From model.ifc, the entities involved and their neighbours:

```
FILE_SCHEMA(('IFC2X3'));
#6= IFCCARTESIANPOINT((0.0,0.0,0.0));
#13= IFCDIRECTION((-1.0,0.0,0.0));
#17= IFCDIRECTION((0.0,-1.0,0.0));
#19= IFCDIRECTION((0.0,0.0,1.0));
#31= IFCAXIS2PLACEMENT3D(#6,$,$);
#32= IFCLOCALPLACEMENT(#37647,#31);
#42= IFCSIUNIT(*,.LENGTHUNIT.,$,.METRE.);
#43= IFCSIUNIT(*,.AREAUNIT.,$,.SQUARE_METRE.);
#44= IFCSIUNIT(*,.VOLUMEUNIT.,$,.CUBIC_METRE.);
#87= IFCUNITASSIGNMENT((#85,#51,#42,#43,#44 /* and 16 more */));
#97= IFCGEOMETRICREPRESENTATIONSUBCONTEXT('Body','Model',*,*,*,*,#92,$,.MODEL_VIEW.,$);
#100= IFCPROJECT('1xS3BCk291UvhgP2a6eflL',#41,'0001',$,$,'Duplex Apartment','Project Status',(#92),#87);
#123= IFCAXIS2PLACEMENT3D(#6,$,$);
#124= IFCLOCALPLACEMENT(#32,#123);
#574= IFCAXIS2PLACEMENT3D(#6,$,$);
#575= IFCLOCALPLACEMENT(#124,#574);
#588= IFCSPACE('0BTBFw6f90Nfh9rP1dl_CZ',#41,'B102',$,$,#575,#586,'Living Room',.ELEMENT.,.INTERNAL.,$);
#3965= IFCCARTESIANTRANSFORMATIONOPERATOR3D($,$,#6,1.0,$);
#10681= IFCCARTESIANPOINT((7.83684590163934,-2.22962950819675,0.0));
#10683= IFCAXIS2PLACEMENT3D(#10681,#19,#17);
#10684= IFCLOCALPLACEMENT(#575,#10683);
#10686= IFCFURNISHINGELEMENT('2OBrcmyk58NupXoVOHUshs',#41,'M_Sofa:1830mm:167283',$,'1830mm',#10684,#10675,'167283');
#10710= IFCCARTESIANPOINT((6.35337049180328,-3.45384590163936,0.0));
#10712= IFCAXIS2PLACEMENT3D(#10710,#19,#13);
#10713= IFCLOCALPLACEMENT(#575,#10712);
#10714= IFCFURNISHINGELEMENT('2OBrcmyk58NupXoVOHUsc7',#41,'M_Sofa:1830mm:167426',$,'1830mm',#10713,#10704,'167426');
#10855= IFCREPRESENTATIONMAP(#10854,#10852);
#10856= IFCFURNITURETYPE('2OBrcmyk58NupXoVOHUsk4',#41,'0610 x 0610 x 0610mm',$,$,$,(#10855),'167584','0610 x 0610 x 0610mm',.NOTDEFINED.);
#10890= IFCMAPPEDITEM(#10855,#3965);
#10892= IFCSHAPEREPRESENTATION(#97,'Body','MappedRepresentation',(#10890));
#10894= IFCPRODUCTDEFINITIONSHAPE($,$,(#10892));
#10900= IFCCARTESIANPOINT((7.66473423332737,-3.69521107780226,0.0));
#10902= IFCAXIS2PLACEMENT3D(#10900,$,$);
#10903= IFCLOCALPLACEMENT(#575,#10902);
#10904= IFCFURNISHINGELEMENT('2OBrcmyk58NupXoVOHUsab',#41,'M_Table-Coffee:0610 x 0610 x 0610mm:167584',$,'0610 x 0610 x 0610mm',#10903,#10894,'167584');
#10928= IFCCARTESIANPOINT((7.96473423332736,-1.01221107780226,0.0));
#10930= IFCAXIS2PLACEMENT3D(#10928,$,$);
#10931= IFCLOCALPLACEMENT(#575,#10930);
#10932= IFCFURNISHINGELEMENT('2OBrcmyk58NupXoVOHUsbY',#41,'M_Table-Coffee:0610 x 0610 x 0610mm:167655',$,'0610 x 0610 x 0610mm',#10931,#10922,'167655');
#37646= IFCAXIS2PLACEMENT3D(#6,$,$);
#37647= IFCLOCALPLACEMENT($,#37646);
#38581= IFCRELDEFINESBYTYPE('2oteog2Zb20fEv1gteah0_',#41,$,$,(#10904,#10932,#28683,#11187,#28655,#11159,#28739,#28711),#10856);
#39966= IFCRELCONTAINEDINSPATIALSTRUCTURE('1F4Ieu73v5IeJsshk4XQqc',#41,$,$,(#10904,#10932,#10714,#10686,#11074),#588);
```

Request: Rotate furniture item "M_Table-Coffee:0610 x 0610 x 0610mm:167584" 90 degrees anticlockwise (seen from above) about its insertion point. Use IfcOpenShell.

```python
import ifcopenshell
import ifcopenshell.api.geometry
import ifcopenshell.util.placement

model = ifcopenshell.open("model.ifc")

item = model.by_guid("2OBrcmyk58NupXoVOHUsab")
matrix = ifcopenshell.util.placement.get_local_placement(item.ObjectPlacement)
matrix = matrix @ ifcopenshell.util.placement.rotation(90, "Z")
ifcopenshell.api.geometry.edit_object_placement(model, product=item, matrix=matrix, is_si=False)

print(ifcopenshell.util.placement.get_local_placement(item.ObjectPlacement).round(3) + 0.0)

model.write("model_edited.ifc")
```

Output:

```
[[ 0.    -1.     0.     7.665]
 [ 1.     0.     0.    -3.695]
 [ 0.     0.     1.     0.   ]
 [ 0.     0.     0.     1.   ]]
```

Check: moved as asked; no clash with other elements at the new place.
